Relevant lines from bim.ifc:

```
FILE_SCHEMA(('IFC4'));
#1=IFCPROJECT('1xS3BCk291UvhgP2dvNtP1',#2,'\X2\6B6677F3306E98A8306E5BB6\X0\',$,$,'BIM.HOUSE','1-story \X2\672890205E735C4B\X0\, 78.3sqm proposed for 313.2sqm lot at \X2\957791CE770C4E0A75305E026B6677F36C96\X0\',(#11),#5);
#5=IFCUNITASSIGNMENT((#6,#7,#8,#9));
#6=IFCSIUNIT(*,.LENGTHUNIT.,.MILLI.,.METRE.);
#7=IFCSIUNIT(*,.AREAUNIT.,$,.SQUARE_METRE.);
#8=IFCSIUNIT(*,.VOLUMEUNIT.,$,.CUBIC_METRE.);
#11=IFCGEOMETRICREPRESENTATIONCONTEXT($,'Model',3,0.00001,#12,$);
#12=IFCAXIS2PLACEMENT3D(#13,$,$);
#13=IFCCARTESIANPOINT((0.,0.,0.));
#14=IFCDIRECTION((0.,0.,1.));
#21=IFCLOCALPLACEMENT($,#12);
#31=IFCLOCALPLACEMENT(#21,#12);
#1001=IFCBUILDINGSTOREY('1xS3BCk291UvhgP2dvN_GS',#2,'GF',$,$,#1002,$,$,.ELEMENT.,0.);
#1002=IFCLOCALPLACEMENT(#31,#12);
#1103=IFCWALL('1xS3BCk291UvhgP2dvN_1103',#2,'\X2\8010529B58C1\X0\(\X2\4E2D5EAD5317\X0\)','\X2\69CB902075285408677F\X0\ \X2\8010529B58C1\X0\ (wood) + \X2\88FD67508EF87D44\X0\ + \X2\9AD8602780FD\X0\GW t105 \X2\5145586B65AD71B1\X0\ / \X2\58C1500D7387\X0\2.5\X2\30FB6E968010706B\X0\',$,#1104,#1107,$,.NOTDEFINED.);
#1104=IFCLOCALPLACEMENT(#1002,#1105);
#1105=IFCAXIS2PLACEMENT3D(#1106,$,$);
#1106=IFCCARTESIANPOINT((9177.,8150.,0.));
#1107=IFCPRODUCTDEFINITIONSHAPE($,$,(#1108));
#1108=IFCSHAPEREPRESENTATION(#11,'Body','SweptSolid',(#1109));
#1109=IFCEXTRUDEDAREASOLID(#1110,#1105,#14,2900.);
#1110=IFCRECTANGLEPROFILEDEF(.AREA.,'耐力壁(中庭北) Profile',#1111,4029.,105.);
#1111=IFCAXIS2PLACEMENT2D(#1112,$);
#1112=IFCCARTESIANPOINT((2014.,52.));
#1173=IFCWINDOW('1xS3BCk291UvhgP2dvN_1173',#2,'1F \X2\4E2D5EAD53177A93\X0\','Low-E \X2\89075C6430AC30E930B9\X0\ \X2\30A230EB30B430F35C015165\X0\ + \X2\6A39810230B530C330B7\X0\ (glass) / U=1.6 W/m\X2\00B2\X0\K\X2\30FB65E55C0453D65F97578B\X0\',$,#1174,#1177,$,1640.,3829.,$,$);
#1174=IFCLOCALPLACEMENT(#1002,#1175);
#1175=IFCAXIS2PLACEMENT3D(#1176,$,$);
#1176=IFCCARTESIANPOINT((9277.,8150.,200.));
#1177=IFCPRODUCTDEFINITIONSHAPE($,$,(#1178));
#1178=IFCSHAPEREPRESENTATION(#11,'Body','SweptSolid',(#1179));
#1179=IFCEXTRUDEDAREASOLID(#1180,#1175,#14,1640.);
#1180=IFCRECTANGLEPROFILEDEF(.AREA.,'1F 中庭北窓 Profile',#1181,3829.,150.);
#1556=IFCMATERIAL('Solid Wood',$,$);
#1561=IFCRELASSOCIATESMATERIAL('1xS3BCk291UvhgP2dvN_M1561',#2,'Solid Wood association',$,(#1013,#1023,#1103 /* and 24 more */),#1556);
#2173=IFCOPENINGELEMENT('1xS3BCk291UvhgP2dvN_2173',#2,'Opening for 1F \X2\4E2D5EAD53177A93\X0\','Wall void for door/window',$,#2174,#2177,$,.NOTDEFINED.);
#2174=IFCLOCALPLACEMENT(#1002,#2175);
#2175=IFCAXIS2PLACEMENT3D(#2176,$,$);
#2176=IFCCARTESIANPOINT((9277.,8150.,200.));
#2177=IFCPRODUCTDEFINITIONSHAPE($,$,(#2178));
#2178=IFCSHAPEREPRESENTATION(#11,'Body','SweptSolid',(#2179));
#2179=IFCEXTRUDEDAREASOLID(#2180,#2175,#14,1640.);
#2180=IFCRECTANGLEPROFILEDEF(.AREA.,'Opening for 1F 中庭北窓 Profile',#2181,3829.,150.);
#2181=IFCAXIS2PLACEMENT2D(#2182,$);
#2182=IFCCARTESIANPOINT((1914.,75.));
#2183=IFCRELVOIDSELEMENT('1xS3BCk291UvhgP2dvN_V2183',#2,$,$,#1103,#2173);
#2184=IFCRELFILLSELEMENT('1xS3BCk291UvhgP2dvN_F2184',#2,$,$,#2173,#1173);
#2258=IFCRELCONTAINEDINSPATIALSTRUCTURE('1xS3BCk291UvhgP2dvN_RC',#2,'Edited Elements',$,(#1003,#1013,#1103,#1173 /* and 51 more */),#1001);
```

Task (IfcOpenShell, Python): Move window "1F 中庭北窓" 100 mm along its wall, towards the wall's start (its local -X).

```python
import ifcopenshell
import ifcopenshell.api.geometry
import ifcopenshell.util.placement
import ifcopenshell.util.unit

model = ifcopenshell.open("bim.ifc")
unit_scale = ifcopenshell.util.unit.calculate_unit_scale(model)

window = model.by_guid("1xS3BCk291UvhgP2dvN_1173")
opening = window.FillsVoids[0].RelatingOpeningElement
wall = opening.VoidsElements[0].RelatingBuildingElement

wall_matrix = ifcopenshell.util.placement.get_local_placement(wall.ObjectPlacement)
shift = wall_matrix[:3, 0] * -0.1 / unit_scale
before = ifcopenshell.util.placement.get_local_placement(window.ObjectPlacement)[:3, 3].copy()

# The window is not placed relative to its opening, so move both.
for product in (opening, window):
    matrix = ifcopenshell.util.placement.get_local_placement(product.ObjectPlacement)
    matrix[:3, 3] += shift
    ifcopenshell.api.geometry.edit_object_placement(model, product=product, matrix=matrix, is_si=False)

after = ifcopenshell.util.placement.get_local_placement(window.ObjectPlacement)[:3, 3]
print("window moved by", (after - before).round(3) + 0.0)

model.write("bim_updated.ifc")
```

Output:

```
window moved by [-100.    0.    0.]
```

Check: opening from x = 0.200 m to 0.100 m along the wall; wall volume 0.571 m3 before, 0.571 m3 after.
